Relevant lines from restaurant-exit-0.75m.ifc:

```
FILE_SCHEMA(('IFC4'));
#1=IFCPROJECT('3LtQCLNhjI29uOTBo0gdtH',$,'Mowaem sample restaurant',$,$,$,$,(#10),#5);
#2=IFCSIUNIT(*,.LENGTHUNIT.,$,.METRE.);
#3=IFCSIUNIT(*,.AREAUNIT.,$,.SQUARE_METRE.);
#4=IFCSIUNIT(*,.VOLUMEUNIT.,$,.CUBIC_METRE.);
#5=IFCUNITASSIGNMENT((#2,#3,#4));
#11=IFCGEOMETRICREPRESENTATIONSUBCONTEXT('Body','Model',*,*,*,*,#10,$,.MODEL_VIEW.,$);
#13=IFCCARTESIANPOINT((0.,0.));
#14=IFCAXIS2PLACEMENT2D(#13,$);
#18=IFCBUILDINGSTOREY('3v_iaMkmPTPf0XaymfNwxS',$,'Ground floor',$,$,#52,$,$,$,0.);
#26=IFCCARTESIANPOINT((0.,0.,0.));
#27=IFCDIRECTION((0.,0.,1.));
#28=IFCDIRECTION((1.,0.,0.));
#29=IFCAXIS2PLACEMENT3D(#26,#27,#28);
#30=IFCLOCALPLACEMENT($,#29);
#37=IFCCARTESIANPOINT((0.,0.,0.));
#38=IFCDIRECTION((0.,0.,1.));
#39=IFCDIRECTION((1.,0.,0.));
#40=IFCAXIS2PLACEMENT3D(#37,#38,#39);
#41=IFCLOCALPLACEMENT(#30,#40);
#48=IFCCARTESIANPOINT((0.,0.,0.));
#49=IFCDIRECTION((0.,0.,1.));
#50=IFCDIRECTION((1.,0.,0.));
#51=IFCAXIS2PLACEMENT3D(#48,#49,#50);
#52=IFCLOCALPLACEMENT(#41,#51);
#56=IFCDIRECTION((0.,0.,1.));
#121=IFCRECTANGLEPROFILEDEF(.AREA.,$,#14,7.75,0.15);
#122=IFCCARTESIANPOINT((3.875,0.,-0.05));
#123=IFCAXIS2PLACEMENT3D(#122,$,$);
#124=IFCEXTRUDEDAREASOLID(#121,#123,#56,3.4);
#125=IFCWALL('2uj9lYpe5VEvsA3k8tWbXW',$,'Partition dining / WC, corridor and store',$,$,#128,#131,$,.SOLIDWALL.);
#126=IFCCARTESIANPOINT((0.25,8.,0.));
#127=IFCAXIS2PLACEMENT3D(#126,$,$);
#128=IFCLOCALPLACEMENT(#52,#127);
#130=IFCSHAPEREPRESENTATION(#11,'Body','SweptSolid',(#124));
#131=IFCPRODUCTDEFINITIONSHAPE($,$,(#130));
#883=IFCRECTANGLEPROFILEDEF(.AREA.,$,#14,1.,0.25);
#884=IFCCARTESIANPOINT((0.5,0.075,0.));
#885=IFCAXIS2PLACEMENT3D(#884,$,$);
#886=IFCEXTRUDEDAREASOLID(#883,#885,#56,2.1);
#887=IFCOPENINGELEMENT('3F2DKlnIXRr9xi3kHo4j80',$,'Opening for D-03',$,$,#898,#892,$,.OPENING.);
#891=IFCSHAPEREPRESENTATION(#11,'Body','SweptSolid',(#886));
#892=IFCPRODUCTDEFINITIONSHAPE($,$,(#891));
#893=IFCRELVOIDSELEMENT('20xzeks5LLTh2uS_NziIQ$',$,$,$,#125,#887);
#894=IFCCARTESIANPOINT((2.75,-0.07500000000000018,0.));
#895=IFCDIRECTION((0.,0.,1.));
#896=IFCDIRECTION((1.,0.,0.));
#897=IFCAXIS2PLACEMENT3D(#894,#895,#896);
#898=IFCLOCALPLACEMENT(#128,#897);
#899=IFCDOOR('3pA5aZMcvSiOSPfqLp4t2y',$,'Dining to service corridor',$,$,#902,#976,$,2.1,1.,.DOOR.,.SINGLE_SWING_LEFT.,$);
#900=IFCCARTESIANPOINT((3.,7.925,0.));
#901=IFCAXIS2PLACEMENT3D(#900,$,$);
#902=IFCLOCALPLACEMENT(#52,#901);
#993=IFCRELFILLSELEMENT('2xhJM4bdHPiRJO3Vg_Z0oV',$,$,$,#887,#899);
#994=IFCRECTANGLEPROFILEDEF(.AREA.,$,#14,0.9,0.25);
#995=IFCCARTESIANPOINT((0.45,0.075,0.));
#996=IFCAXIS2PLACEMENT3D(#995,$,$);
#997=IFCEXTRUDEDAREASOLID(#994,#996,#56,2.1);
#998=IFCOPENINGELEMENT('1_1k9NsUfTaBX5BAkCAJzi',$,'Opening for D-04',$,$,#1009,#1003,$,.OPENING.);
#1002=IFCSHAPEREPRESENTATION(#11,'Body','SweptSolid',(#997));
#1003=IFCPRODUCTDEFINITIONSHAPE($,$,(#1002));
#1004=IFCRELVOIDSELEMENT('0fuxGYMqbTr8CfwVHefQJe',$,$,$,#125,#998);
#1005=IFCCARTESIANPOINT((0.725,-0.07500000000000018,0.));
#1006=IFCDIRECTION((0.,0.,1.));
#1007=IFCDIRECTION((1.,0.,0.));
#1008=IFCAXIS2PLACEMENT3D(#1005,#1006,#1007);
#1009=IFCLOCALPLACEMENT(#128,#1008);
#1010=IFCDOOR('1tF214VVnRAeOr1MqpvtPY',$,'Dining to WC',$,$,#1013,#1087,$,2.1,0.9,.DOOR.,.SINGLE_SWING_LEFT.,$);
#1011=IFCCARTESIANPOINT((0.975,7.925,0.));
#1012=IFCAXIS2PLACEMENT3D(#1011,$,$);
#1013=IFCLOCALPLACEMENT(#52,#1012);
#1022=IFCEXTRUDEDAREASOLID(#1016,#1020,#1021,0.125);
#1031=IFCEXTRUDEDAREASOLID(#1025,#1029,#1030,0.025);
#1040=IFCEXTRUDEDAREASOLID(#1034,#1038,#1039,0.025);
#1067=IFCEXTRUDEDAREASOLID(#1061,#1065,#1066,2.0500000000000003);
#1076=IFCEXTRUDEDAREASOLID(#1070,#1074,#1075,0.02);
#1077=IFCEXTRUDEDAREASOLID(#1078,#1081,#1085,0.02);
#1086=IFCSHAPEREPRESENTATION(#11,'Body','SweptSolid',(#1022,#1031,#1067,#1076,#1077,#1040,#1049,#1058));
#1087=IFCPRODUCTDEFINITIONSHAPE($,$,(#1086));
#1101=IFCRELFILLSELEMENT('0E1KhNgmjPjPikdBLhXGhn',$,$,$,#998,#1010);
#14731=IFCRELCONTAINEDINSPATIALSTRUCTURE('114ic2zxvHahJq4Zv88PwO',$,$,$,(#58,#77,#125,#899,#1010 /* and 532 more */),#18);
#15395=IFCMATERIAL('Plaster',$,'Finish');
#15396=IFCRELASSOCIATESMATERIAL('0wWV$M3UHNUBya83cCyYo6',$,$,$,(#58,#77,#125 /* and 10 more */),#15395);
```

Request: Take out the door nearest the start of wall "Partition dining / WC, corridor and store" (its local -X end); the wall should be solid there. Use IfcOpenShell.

```python
import ifcopenshell
import ifcopenshell.api.feature
import ifcopenshell.api.root
import ifcopenshell.geom
import ifcopenshell.util.shape

model = ifcopenshell.open("restaurant-exit-0.75m.ifc")
settings = ifcopenshell.geom.settings()


def volume(element):
    """Net volume in cubic metres, openings subtracted."""
    shape = ifcopenshell.geom.create_shape(settings, element)
    return ifcopenshell.util.shape.get_volume(shape.geometry)


door = model.by_guid("1tF214VVnRAeOr1MqpvtPY")
opening = door.FillsVoids[0].RelatingOpeningElement
wall = opening.VoidsElements[0].RelatingBuildingElement
before = volume(wall)

ifcopenshell.api.root.remove_product(model, product=door)
ifcopenshell.api.feature.remove_feature(model, feature=opening)

after = volume(wall)

print(f"wall volume {before:.3f} -> {after:.3f} m3")

model.write("restaurant-exit-0.75m_rev.ifc")
```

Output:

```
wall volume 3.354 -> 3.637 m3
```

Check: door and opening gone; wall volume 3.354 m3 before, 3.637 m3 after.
